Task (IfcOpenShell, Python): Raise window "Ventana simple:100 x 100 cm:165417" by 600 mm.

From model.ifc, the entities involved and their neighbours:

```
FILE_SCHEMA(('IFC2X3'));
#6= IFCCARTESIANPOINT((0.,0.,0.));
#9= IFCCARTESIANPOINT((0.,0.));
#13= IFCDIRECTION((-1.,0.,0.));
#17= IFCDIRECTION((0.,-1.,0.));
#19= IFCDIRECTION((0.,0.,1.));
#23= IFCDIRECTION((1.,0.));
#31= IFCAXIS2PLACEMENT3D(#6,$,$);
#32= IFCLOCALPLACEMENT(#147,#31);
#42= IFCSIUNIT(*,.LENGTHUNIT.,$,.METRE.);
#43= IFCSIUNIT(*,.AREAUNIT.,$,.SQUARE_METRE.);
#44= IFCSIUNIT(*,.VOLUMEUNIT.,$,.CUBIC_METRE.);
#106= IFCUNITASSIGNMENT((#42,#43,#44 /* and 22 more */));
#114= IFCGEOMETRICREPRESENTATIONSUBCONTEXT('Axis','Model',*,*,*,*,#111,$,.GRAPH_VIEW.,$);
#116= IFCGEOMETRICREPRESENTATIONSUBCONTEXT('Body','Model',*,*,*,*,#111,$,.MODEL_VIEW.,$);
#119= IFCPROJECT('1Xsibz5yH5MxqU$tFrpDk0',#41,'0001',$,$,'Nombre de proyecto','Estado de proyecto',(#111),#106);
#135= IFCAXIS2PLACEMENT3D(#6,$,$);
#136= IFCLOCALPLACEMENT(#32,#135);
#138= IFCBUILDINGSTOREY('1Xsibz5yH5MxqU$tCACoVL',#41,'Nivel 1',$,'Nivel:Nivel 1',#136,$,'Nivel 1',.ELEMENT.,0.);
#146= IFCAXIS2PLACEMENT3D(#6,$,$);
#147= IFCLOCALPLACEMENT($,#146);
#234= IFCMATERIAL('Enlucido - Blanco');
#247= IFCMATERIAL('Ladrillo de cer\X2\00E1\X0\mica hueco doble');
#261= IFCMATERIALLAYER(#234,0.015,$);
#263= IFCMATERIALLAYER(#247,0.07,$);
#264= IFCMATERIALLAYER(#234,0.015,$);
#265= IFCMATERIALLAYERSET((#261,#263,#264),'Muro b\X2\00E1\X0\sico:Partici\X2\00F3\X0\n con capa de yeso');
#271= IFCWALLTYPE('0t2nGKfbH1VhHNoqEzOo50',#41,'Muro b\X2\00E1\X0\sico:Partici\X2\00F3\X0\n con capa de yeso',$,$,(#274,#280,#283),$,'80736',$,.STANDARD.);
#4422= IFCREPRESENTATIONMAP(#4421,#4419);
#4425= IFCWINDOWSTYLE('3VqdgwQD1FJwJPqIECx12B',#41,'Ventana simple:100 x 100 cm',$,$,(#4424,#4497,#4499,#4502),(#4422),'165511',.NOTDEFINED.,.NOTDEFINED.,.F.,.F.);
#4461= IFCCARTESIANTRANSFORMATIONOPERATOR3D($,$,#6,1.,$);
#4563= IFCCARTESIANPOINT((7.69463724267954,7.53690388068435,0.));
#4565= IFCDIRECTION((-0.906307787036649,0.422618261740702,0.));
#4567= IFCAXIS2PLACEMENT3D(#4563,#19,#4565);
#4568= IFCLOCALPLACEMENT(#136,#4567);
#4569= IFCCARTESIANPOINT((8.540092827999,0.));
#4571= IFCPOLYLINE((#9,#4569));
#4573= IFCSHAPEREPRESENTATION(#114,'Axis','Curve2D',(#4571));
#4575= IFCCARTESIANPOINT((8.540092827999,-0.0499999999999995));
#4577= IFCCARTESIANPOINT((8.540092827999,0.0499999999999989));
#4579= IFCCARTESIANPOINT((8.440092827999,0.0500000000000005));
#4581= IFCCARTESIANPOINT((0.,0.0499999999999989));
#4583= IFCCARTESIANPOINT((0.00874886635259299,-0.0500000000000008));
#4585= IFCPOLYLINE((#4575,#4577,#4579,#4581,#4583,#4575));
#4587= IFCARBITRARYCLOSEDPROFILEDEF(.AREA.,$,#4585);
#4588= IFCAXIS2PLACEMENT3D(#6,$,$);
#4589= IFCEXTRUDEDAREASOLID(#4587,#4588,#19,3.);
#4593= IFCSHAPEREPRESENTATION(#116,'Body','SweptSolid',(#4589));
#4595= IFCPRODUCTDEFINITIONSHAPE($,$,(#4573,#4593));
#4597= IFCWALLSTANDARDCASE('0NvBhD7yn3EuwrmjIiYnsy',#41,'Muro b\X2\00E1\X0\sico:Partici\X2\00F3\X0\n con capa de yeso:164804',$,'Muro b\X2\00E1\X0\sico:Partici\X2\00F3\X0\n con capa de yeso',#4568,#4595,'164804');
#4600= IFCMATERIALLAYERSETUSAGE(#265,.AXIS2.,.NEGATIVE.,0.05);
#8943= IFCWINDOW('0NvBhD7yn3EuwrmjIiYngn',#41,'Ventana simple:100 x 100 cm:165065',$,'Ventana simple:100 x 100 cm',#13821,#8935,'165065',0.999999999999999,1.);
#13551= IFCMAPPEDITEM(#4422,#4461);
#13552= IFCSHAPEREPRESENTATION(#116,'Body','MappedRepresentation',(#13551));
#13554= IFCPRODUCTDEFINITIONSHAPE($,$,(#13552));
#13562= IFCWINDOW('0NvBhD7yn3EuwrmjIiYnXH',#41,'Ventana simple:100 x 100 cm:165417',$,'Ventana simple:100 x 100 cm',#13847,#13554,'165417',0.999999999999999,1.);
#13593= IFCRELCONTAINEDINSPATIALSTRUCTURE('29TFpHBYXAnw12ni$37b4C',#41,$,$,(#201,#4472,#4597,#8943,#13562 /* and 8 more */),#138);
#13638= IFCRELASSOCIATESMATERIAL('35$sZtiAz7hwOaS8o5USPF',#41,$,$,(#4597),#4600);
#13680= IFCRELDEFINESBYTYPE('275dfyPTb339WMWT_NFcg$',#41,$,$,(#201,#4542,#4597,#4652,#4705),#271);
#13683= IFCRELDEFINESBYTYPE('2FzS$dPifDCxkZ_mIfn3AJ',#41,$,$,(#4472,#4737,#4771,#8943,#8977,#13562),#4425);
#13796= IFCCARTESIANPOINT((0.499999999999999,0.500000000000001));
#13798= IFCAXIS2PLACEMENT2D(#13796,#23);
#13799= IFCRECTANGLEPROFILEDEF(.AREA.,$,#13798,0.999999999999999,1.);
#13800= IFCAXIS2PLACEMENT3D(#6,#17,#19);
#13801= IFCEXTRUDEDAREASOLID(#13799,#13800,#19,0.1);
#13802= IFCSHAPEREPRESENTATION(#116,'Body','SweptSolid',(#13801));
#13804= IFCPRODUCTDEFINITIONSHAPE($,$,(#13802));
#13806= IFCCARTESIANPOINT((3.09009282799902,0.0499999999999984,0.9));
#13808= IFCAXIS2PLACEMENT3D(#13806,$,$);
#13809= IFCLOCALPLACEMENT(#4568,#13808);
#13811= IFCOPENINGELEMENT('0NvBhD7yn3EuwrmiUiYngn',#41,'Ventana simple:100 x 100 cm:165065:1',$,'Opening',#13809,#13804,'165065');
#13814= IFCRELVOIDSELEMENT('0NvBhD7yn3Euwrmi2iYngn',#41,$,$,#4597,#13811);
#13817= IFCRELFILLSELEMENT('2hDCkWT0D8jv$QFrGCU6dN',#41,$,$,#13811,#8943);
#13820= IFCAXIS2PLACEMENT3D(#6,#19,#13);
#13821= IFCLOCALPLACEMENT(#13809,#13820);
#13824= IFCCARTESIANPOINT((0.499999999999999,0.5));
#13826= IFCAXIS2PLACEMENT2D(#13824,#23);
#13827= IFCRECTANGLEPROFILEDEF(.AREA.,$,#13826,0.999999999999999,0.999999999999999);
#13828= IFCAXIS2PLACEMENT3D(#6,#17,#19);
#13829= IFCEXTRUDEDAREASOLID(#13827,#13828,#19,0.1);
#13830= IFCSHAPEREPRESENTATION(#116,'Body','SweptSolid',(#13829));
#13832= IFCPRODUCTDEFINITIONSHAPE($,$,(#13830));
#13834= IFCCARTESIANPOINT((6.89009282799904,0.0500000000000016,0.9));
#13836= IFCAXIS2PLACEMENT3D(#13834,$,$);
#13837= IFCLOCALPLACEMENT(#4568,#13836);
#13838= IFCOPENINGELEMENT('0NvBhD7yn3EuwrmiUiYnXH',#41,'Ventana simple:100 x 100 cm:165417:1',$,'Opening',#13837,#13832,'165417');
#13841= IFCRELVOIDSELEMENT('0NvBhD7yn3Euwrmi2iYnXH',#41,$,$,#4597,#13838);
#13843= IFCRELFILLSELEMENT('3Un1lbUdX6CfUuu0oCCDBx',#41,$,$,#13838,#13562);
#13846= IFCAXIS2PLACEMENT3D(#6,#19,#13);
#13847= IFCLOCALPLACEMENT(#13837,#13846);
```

```python
import numpy as np
import ifcopenshell
import ifcopenshell.api.geometry
import ifcopenshell.util.placement
import ifcopenshell.util.unit

model = ifcopenshell.open("model.ifc")
unit_scale = ifcopenshell.util.unit.calculate_unit_scale(model)

window = model.by_id(13562)
opening = window.FillsVoids[0].RelatingOpeningElement
dz = 0.6

shift = np.array([0.0, 0.0, dz])
# The window is placed relative to its opening, so it follows when the opening moves.
matrix = ifcopenshell.util.placement.get_local_placement(opening.ObjectPlacement)
matrix[:3, 3] += shift
ifcopenshell.api.geometry.edit_object_placement(
    model, product=opening, matrix=matrix, is_si=False, should_transform_children=True
)

print(f"moved by {dz * unit_scale:+.3f} m")

model.write("model-out.ifc")
```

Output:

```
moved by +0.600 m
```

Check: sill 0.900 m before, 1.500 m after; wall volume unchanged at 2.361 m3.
